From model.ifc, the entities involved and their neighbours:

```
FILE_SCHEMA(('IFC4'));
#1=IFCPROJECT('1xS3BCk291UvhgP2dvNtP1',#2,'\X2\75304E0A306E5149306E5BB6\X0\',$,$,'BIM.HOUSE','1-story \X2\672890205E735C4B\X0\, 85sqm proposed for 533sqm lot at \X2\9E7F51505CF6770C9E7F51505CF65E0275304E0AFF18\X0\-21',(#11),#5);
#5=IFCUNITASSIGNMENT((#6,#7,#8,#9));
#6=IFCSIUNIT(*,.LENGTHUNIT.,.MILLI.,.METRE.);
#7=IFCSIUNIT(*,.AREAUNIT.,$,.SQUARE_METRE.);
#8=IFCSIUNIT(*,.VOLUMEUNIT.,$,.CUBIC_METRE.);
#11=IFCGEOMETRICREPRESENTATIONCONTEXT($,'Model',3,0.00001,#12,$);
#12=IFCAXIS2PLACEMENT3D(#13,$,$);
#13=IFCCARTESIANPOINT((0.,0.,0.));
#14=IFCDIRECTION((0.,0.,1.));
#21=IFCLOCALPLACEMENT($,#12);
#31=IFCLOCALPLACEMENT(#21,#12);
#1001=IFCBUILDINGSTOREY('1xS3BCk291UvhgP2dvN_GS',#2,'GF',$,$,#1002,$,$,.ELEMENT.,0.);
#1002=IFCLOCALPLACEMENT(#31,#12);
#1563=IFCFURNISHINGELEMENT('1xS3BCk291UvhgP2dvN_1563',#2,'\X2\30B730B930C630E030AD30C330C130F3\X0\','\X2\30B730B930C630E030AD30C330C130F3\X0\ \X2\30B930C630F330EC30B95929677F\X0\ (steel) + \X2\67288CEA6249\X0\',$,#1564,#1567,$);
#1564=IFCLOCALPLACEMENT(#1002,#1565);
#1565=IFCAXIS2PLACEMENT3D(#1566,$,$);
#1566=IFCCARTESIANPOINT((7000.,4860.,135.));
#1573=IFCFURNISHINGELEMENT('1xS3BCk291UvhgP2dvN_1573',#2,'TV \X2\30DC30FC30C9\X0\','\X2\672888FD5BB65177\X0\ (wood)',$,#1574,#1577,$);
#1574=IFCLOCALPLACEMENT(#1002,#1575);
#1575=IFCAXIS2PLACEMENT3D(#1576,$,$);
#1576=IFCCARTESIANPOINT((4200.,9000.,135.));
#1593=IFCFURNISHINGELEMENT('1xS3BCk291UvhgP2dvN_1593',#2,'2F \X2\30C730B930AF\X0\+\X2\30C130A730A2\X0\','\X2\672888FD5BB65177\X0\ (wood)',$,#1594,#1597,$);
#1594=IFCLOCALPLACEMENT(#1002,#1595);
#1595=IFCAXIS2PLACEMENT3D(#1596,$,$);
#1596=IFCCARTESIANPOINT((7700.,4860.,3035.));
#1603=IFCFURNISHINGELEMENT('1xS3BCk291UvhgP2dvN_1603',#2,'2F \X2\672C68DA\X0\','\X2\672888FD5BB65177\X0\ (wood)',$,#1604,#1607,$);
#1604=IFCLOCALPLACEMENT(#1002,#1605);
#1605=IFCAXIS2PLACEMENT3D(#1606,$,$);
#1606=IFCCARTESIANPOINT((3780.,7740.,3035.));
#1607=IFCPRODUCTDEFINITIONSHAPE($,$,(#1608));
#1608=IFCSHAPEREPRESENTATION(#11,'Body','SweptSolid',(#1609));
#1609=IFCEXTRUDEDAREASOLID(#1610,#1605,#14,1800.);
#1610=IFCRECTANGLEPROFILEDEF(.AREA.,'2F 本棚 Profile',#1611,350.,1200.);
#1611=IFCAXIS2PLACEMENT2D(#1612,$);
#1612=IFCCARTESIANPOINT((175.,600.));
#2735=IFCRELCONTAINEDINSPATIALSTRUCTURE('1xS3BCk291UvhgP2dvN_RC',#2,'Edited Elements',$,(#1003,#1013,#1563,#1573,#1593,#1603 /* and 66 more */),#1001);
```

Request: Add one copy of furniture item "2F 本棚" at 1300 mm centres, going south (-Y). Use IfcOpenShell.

```python
import numpy as np
import ifcopenshell
import ifcopenshell.api.geometry
import ifcopenshell.api.root
import ifcopenshell.util.element
import ifcopenshell.util.placement
import ifcopenshell.util.unit

model = ifcopenshell.open("model.ifc")
unit_scale = ifcopenshell.util.unit.calculate_unit_scale(model)


def reuse_history(source, copy):
    """copy_class also copies each property set's owner history, people and application; keep the originals."""
    for rel in copy.IsDefinedBy:
        if rel.is_a("IfcRelDefinesByProperties") and (history := rel.RelatingPropertyDefinition.OwnerHistory):
            rel.RelatingPropertyDefinition.OwnerHistory = source.OwnerHistory
            ifcopenshell.util.element.remove_deep2(model, history)


source = model.by_id(1603)
base = ifcopenshell.util.placement.get_local_placement(source.ObjectPlacement)
step = np.array([0.0, -1.0, 0.0]) * 1.3 / unit_scale

for i in range(1, 2):
    copy = ifcopenshell.api.root.copy_class(model, product=source)
    copy.Representation = ifcopenshell.util.element.copy_deep(
        model, source.Representation, exclude=["IfcGeometricRepresentationContext", "IfcRepresentationMap"]
    )
    reuse_history(source, copy)
    matrix = base.copy()
    matrix[:3, 3] += i * step
    print("added at", matrix[:3, 3].round(3) + 0.0)
    ifcopenshell.api.geometry.edit_object_placement(model, product=copy, matrix=matrix, is_si=False)

model.write("model_updated.ifc")
```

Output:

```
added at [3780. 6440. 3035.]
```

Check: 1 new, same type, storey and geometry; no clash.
